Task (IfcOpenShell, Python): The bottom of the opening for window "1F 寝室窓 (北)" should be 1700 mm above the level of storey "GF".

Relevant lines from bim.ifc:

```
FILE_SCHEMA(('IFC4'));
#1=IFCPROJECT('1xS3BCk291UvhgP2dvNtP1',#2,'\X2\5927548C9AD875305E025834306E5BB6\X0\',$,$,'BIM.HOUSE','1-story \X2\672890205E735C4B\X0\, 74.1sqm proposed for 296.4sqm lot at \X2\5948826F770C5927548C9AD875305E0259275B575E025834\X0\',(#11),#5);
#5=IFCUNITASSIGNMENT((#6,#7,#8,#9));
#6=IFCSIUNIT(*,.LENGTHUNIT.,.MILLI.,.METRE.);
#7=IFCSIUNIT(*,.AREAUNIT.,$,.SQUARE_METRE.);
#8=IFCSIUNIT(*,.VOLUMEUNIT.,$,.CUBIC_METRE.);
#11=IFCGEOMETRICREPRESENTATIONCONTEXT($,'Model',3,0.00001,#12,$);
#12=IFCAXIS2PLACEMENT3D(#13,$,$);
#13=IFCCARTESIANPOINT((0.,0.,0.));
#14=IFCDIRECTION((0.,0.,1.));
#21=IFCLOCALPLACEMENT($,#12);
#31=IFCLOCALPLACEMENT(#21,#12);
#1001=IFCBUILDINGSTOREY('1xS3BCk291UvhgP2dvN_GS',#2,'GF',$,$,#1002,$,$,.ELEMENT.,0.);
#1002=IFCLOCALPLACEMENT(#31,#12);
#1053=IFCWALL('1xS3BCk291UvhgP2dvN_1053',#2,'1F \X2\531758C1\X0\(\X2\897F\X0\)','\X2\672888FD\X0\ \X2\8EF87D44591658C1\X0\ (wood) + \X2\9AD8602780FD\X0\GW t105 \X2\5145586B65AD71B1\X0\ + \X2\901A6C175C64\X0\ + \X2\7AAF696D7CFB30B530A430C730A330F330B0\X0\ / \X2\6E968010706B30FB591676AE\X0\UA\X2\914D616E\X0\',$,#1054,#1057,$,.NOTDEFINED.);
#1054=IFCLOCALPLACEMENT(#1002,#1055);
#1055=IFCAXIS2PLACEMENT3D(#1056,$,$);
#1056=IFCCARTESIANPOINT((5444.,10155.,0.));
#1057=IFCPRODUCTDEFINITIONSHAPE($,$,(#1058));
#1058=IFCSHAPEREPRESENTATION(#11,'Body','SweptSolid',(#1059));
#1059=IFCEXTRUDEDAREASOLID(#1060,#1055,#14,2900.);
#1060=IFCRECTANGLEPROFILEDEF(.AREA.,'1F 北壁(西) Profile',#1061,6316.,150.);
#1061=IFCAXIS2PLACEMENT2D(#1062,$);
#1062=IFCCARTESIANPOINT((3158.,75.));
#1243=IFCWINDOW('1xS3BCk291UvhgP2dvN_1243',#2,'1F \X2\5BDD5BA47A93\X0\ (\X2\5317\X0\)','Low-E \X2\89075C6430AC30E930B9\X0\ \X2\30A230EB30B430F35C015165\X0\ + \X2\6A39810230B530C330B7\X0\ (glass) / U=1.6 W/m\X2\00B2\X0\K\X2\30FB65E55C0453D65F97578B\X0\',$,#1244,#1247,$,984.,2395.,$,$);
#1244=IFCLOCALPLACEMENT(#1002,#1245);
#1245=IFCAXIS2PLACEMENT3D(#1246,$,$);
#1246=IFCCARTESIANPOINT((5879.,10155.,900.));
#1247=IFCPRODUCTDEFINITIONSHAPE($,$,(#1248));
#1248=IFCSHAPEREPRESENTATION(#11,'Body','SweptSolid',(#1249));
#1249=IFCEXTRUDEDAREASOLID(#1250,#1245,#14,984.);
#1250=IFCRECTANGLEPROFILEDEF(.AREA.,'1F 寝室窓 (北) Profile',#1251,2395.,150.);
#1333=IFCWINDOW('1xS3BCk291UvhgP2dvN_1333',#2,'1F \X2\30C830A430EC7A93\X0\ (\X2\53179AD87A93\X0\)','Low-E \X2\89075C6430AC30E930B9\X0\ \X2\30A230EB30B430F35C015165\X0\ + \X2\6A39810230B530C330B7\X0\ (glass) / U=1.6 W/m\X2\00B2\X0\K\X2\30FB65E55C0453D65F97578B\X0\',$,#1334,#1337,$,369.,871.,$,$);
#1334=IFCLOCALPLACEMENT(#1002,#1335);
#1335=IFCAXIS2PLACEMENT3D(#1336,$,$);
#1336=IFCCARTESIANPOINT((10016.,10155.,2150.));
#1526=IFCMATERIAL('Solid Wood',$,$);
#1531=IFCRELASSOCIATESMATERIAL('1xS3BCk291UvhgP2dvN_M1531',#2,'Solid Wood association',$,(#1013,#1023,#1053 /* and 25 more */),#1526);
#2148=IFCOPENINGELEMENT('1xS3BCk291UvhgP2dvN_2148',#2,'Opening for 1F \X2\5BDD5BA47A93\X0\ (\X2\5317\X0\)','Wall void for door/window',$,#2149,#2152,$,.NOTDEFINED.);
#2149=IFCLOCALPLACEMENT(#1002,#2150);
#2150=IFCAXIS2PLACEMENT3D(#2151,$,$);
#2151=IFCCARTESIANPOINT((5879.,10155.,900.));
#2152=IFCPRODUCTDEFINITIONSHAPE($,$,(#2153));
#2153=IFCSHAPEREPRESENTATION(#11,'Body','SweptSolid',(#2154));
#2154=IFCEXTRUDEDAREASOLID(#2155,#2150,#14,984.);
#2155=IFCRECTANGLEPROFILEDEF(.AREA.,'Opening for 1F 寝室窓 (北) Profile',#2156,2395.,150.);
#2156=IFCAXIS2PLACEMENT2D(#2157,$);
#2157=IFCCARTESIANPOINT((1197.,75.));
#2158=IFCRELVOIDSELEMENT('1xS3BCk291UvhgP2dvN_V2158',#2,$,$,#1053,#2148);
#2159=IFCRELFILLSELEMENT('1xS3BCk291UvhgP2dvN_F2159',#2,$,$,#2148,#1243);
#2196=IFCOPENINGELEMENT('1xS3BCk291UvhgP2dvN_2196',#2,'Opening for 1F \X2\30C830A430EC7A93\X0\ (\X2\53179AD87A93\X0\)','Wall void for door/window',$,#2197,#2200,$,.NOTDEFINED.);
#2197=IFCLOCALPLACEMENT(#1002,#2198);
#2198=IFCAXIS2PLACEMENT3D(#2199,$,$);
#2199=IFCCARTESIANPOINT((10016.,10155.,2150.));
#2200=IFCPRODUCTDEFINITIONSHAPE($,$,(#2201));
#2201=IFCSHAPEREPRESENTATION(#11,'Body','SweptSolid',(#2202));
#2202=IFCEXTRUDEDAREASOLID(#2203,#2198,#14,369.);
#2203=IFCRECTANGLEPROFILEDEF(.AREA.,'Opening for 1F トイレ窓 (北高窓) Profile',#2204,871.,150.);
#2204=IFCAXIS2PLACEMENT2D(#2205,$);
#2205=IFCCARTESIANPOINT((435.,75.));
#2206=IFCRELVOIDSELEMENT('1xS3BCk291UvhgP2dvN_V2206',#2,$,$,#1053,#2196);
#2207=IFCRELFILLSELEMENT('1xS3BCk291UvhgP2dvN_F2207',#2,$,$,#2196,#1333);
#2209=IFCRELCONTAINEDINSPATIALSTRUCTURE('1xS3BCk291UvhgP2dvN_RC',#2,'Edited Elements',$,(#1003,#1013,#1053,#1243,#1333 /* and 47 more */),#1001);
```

```python
import numpy as np
import ifcopenshell
import ifcopenshell.api.geometry
import ifcopenshell.geom
import ifcopenshell.util.element
import ifcopenshell.util.placement
import ifcopenshell.util.shape
import ifcopenshell.util.unit

model = ifcopenshell.open("bim.ifc")
unit_scale = ifcopenshell.util.unit.calculate_unit_scale(model)

window = model.by_guid("1xS3BCk291UvhgP2dvN_1243")
opening = window.FillsVoids[0].RelatingOpeningElement
storey = ifcopenshell.util.element.get_container(window, ifc_class="IfcBuildingStorey")
level = ifcopenshell.util.placement.get_local_placement(storey.ObjectPlacement)[2, 3]

# The opening's origin need not be at the sill, so measure its lowest point.
shape = ifcopenshell.geom.create_shape(ifcopenshell.geom.settings(), opening)
bottom = ifcopenshell.util.shape.get_shape_bottom_elevation(shape, shape.geometry) / unit_scale
dz = level + 1.7 / unit_scale - bottom

shift = np.array([0.0, 0.0, dz])
# The window is not placed relative to its opening, so move both.
for product in (opening, window):
    matrix = ifcopenshell.util.placement.get_local_placement(product.ObjectPlacement)
    matrix[:3, 3] += shift
    ifcopenshell.api.geometry.edit_object_placement(model, product=product, matrix=matrix, is_si=False)

print(f"moved by {dz * unit_scale:+.3f} m")

model.write("bim_updated.ifc")
```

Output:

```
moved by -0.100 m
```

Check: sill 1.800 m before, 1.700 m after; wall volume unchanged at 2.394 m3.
